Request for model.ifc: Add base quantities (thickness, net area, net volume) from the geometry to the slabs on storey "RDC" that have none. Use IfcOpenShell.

First a look at what the model holds.

```python
import ifcopenshell
import ifcopenshell.util.element
import ifcopenshell.util.unit

model = ifcopenshell.open("model.ifc")
print(model.schema)
for unit_type in ("LENGTHUNIT", "AREAUNIT", "VOLUMEUNIT"):
    print(unit_type, ifcopenshell.util.unit.calculate_unit_scale(model, unit_type))
storey = next(s for s in model.by_type("IfcBuildingStorey") if s.Name == "RDC")
slabs = [e for e in ifcopenshell.util.element.get_decomposition(storey) if e.is_a("IfcSlab")]
for e in sorted(slabs, key=lambda e: e.id()):
    print(e.id(), e.is_a(), e.Name, list(ifcopenshell.util.element.get_psets(e, qtos_only=True)), sep=" | ")
```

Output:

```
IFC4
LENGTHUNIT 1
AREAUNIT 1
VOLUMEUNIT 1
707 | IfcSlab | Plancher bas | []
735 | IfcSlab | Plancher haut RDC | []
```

```python
import ifcopenshell
import ifcopenshell.api.pset
import ifcopenshell.geom
import ifcopenshell.util.element
import ifcopenshell.util.shape
import ifcopenshell.util.unit

model = ifcopenshell.open("model.ifc")
unit_scale = ifcopenshell.util.unit.calculate_unit_scale(model)
area_scale = ifcopenshell.util.unit.calculate_unit_scale(model, "AREAUNIT")
volume_scale = ifcopenshell.util.unit.calculate_unit_scale(model, "VOLUMEUNIT")
settings = ifcopenshell.geom.settings()

storey = next(s for s in model.by_type("IfcBuildingStorey") if s.Name == "RDC")
slabs = [e for e in ifcopenshell.util.element.get_decomposition(storey) if e.is_a("IfcSlab")]

for e in sorted(slabs, key=lambda e: e.id()):
    if ifcopenshell.util.element.get_psets(e, qtos_only=True, should_inherit=False):
        continue
    # Geometry comes back in metres, in the element's own axes.
    shape = ifcopenshell.geom.create_shape(settings, e)
    values = {
        "Width": ifcopenshell.util.shape.get_z(shape.geometry) / unit_scale,
        "NetArea": ifcopenshell.util.shape.get_footprint_area(shape.geometry) / area_scale,
        "NetVolume": ifcopenshell.util.shape.get_volume(shape.geometry) / volume_scale,
    }
    qto = ifcopenshell.api.pset.add_qto(model, product=e, name="Qto_SlabBaseQuantities")
    ifcopenshell.api.pset.edit_qto(model, qto=qto, properties=values)
    print(e.id(), {k: round(v, 3) for k, v in values.items()})

model.write("model_v2.ifc")
```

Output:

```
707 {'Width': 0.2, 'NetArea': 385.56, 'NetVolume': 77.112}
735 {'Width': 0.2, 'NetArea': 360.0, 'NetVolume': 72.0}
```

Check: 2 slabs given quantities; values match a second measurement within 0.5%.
